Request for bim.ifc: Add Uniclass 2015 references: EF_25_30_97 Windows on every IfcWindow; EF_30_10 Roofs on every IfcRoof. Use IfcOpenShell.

First a look at what the model holds.

```python
import ifcopenshell

model = ifcopenshell.open("bim.ifc")
print(model.schema)
print("classifications:", [c.Name for c in model.by_type("IfcClassification")])
for ifc_class in ("IfcDoor", "IfcRoof", "IfcStair", "IfcWall", "IfcWindow"):
    print(ifc_class, len(model.by_type(ifc_class)))
```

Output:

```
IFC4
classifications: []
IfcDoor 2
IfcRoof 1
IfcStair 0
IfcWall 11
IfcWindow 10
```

```python
import ifcopenshell
import ifcopenshell.api.classification

model = ifcopenshell.open("bim.ifc")

system = ifcopenshell.api.classification.add_classification(model, classification="Uniclass 2015")

codes = {
    "IfcWindow": ("EF_25_30_97", "Windows"),
    "IfcRoof": ("EF_30_10", "Roofs"),
}
for ifc_class, (code, name) in codes.items():
    products = model.by_type(ifc_class)
    ifcopenshell.api.classification.add_reference(
        model, products=products, classification=system, identification=code, name=name
    )
    print(code, len(products))

model.write("bim_rev.ifc")
```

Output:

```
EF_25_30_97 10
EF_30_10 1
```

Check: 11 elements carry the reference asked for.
